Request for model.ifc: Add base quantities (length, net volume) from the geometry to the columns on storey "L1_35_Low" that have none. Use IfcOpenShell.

First a look at what the model holds.

```python
import ifcopenshell
import ifcopenshell.util.element
import ifcopenshell.util.unit

model = ifcopenshell.open("model.ifc")
print(model.schema)
for unit_type in ("LENGTHUNIT", "AREAUNIT", "VOLUMEUNIT"):
    print(unit_type, ifcopenshell.util.unit.calculate_unit_scale(model, unit_type))
storey = next(s for s in model.by_type("IfcBuildingStorey") if s.Name == "L1_35_Low")
columns = [e for e in ifcopenshell.util.element.get_decomposition(storey) if e.is_a("IfcColumn")]
for e in sorted(columns, key=lambda e: e.id()):
    print(e.id(), e.is_a(), e.Name, list(ifcopenshell.util.element.get_psets(e, qtos_only=True)), sep=" | ")
```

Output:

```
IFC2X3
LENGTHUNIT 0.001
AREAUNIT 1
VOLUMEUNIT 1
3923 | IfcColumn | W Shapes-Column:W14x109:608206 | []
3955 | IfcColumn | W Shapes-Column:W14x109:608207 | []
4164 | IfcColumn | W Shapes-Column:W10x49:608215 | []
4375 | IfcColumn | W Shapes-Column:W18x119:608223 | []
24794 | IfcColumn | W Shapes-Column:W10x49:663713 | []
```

```python
import ifcopenshell
import ifcopenshell.api.pset
import ifcopenshell.geom
import ifcopenshell.util.element
import ifcopenshell.util.shape
import ifcopenshell.util.unit

model = ifcopenshell.open("model.ifc")
unit_scale = ifcopenshell.util.unit.calculate_unit_scale(model)
volume_scale = ifcopenshell.util.unit.calculate_unit_scale(model, "VOLUMEUNIT")
settings = ifcopenshell.geom.settings()

storey = next(s for s in model.by_type("IfcBuildingStorey") if s.Name == "L1_35_Low")
columns = [e for e in ifcopenshell.util.element.get_decomposition(storey) if e.is_a("IfcColumn")]

for e in sorted(columns, key=lambda e: e.id()):
    if ifcopenshell.util.element.get_psets(e, qtos_only=True, should_inherit=False):
        continue
    # Geometry comes back in metres, in the element's own axes.
    shape = ifcopenshell.geom.create_shape(settings, e)
    values = {
        "Length": ifcopenshell.util.shape.get_z(shape.geometry) / unit_scale,
        "NetVolume": ifcopenshell.util.shape.get_volume(shape.geometry) / volume_scale,
    }
    qto = ifcopenshell.api.pset.add_qto(model, product=e, name="BaseQuantities")
    ifcopenshell.api.pset.edit_qto(model, qto=qto, properties=values)
    print(e.id(), {k: round(v, 3) for k, v in values.items()})

model.write("model_rev.ifc")
```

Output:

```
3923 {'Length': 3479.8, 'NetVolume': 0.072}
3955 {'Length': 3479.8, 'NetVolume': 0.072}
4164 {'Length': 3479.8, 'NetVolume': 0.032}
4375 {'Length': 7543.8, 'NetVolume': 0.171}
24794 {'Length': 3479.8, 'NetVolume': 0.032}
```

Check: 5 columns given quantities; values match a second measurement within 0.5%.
